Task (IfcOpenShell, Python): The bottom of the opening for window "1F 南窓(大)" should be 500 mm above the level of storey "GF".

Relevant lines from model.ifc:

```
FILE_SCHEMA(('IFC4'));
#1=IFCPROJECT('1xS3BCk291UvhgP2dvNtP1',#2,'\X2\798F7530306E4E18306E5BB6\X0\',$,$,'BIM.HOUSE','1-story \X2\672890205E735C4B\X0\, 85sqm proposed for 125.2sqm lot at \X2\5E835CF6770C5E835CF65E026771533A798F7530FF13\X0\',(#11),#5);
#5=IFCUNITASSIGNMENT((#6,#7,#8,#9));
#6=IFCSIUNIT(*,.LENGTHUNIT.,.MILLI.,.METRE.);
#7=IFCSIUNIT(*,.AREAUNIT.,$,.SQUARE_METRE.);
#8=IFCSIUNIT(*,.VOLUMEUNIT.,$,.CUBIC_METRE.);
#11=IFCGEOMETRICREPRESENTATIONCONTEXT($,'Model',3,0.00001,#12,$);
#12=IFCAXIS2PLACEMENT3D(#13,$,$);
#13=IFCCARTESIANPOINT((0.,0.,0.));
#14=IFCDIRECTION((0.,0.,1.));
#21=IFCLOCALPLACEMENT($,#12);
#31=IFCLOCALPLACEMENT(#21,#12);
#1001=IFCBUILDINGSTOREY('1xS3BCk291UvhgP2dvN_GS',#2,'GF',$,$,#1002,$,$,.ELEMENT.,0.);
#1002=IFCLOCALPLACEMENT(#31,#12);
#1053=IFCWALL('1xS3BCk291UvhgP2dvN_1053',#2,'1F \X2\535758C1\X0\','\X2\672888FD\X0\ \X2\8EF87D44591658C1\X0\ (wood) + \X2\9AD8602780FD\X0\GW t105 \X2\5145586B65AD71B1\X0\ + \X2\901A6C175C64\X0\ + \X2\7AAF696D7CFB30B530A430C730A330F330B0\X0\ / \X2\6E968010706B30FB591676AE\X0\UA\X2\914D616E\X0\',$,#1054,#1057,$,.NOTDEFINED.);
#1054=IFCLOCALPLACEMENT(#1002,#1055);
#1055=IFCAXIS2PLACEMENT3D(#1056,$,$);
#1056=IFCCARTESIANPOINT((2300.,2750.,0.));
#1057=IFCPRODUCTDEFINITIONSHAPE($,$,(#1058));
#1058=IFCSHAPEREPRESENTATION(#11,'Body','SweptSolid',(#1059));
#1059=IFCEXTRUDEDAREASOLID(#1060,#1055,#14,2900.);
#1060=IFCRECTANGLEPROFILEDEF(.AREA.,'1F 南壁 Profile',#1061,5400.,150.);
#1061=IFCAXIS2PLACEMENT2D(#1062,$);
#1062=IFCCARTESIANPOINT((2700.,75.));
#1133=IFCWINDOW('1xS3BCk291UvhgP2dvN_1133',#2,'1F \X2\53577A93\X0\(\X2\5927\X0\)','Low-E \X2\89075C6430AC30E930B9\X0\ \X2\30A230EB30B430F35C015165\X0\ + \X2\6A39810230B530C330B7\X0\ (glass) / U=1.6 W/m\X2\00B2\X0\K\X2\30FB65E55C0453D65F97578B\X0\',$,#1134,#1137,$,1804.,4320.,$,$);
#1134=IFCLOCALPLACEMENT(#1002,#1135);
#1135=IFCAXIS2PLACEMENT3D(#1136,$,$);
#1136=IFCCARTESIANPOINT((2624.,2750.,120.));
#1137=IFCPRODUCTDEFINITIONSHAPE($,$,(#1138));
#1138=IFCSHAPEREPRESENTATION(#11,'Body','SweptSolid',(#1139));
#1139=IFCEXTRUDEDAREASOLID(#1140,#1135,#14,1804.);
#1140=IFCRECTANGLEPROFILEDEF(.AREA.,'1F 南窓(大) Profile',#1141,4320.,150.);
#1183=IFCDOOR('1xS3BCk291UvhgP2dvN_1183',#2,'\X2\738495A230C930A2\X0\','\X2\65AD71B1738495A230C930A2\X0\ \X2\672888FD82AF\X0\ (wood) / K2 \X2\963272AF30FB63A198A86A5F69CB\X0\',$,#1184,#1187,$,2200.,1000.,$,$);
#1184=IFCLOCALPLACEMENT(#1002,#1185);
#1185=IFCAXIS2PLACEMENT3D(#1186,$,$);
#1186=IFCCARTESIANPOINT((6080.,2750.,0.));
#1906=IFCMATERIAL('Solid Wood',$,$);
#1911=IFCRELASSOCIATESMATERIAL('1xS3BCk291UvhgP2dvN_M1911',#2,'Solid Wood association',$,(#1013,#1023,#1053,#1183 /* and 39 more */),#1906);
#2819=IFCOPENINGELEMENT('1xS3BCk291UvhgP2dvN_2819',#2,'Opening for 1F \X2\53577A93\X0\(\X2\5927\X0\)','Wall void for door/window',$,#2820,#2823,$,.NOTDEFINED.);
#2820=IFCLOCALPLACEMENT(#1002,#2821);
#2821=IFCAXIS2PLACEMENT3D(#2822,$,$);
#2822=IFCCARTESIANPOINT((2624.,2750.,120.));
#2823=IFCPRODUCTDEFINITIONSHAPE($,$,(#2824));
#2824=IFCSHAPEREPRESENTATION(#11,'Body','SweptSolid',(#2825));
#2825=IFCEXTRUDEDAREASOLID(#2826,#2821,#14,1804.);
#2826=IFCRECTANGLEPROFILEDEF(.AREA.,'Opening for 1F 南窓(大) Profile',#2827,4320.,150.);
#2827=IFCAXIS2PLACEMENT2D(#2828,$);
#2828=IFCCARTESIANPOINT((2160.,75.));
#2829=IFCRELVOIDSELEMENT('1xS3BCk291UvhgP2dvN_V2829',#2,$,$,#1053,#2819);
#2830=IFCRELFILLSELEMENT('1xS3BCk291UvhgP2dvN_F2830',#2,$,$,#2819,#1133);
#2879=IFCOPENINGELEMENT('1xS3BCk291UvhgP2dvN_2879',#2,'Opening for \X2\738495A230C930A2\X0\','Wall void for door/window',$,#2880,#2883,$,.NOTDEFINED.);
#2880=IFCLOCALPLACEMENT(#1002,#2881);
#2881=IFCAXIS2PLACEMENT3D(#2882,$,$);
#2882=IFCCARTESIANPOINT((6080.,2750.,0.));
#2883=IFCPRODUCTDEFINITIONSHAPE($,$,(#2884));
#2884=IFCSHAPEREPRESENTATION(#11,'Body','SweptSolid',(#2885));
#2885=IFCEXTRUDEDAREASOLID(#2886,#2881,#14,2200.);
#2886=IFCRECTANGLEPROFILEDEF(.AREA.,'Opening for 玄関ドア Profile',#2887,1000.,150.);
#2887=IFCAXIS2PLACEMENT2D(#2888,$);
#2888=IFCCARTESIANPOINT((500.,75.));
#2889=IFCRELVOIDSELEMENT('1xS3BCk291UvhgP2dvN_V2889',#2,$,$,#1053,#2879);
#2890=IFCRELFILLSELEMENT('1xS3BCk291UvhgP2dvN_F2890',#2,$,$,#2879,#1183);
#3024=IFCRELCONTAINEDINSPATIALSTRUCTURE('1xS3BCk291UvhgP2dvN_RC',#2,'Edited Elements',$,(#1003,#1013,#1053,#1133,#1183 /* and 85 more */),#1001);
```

```python
import numpy as np
import ifcopenshell
import ifcopenshell.api.geometry
import ifcopenshell.geom
import ifcopenshell.util.element
import ifcopenshell.util.placement
import ifcopenshell.util.shape
import ifcopenshell.util.unit

model = ifcopenshell.open("model.ifc")
unit_scale = ifcopenshell.util.unit.calculate_unit_scale(model)

window = model.by_guid("1xS3BCk291UvhgP2dvN_1133")
opening = window.FillsVoids[0].RelatingOpeningElement
storey = ifcopenshell.util.element.get_container(window, ifc_class="IfcBuildingStorey")
level = ifcopenshell.util.placement.get_local_placement(storey.ObjectPlacement)[2, 3]

# The opening's origin need not be at the sill, so measure its lowest point.
shape = ifcopenshell.geom.create_shape(ifcopenshell.geom.settings(), opening)
bottom = ifcopenshell.util.shape.get_shape_bottom_elevation(shape, shape.geometry) / unit_scale
dz = level + 500.0 - bottom

shift = np.array([0.0, 0.0, dz])
# The window is not placed relative to its opening, so move both.
for product in (opening, window):
    matrix = ifcopenshell.util.placement.get_local_placement(product.ObjectPlacement)
    matrix[:3, 3] += shift
    ifcopenshell.api.geometry.edit_object_placement(model, product=product, matrix=matrix, is_si=False)

print(f"moved by {dz * unit_scale:+.3f} m")

model.write("model_v2.ifc")
```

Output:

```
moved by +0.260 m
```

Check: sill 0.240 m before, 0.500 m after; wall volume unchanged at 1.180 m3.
